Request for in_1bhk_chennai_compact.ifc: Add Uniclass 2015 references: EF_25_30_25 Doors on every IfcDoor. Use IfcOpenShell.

First a look at what the model holds.

```python
import ifcopenshell

model = ifcopenshell.open("in_1bhk_chennai_compact.ifc")
print(model.schema)
print("classifications:", [c.Name for c in model.by_type("IfcClassification")])
for ifc_class in ("IfcDoor", "IfcRoof", "IfcStair", "IfcWall", "IfcWindow"):
    print(ifc_class, len(model.by_type(ifc_class)))
```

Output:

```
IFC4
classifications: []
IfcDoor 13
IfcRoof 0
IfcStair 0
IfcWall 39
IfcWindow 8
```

```python
import ifcopenshell
import ifcopenshell.api.classification

model = ifcopenshell.open("in_1bhk_chennai_compact.ifc")

system = ifcopenshell.api.classification.add_classification(model, classification="Uniclass 2015")

codes = {
    "IfcDoor": ("EF_25_30_25", "Doors"),
}
for ifc_class, (code, name) in codes.items():
    products = model.by_type(ifc_class)
    ifcopenshell.api.classification.add_reference(
        model, products=products, classification=system, identification=code, name=name
    )
    print(code, len(products))

model.write("in_1bhk_chennai_compact_rev.ifc")
```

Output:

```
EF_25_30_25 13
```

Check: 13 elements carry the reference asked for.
